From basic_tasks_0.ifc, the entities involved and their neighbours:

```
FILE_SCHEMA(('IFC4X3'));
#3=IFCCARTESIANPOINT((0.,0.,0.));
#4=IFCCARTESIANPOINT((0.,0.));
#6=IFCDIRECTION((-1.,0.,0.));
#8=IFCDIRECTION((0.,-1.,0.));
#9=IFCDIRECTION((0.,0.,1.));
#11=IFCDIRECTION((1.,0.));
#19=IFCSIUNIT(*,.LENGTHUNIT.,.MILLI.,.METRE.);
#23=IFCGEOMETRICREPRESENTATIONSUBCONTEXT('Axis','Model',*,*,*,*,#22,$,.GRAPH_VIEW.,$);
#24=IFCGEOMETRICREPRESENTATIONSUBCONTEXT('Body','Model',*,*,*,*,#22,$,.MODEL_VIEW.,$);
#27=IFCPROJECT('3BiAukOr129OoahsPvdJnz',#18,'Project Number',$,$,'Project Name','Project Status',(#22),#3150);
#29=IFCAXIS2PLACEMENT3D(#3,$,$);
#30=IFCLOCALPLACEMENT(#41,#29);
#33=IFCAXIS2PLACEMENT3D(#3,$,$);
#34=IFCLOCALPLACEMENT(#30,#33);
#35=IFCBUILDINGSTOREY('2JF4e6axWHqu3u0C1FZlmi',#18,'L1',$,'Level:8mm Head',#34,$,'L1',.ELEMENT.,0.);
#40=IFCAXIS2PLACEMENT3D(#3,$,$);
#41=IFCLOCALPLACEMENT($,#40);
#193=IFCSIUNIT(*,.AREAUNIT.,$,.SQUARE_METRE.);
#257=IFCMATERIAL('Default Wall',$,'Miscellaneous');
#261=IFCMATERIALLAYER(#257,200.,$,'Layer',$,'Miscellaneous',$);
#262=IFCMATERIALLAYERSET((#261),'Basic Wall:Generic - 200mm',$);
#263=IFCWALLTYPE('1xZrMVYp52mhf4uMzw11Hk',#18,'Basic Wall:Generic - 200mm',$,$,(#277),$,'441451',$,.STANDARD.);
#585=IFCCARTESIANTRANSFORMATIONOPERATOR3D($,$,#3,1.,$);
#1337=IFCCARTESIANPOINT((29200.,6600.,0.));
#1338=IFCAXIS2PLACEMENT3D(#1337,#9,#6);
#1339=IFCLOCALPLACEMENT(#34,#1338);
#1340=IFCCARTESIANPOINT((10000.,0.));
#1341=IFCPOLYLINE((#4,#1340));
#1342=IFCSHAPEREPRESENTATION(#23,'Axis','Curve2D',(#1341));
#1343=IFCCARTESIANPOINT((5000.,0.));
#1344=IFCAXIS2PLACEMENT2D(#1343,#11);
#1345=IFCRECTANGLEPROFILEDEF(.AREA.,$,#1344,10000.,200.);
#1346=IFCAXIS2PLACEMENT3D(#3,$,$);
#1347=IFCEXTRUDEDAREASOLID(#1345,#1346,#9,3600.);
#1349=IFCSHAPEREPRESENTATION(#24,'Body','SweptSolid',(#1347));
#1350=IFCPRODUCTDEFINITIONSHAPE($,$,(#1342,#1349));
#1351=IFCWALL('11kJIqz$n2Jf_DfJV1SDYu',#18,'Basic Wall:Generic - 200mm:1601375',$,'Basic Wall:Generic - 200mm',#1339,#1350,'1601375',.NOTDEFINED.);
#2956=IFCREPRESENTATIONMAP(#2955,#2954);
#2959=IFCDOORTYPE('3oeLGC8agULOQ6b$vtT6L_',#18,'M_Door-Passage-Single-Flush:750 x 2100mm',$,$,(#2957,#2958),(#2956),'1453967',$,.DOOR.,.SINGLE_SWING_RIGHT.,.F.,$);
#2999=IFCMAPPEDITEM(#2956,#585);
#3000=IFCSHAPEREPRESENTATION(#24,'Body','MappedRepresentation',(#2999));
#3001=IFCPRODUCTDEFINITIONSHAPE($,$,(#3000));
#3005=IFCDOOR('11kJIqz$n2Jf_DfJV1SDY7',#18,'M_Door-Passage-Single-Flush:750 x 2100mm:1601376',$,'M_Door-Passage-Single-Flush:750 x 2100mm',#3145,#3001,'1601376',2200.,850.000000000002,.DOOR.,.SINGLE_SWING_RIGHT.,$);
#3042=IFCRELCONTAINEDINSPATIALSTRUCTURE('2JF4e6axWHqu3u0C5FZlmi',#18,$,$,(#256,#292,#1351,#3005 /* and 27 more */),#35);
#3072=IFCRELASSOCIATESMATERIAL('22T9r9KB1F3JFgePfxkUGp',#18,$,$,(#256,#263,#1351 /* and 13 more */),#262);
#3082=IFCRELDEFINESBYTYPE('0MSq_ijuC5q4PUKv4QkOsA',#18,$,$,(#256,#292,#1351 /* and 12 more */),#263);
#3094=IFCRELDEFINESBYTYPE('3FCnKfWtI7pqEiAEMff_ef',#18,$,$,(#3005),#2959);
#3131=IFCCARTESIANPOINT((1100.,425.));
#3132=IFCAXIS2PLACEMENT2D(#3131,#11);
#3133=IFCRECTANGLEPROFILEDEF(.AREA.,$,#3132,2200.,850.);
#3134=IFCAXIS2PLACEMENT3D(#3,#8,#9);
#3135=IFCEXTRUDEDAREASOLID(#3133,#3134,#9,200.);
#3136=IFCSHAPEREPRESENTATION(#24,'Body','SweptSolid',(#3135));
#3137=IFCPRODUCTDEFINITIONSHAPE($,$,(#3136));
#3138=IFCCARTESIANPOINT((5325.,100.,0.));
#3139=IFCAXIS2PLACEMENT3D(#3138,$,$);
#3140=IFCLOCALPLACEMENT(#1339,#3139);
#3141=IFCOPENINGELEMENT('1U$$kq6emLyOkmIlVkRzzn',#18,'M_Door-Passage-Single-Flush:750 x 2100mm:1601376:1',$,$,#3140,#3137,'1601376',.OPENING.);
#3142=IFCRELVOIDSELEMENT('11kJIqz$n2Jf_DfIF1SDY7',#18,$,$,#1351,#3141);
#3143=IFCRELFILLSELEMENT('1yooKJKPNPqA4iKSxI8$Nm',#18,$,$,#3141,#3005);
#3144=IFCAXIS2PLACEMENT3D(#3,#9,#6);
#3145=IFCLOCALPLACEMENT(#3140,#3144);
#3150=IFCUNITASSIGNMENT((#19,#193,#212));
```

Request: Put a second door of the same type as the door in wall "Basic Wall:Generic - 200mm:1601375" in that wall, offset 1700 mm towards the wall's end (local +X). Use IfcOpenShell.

```python
import ifcopenshell
import ifcopenshell.api.feature
import ifcopenshell.api.geometry
import ifcopenshell.api.root
import ifcopenshell.geom
import ifcopenshell.util.element
import ifcopenshell.util.placement
import ifcopenshell.util.shape
import ifcopenshell.util.unit

model = ifcopenshell.open("basic_tasks_0.ifc")
unit_scale = ifcopenshell.util.unit.calculate_unit_scale(model)
settings = ifcopenshell.geom.settings()


def volume(element):
    """Net volume in cubic metres, openings subtracted."""
    shape = ifcopenshell.geom.create_shape(settings, element)
    return ifcopenshell.util.shape.get_volume(shape.geometry)


def reuse_history(source, copy):
    """copy_class also copies each property set's owner history, people and application; keep the originals."""
    for rel in copy.IsDefinedBy:
        if rel.is_a("IfcRelDefinesByProperties") and (history := rel.RelatingPropertyDefinition.OwnerHistory):
            rel.RelatingPropertyDefinition.OwnerHistory = source.OwnerHistory
            ifcopenshell.util.element.remove_deep2(model, history)


door = model.by_guid("11kJIqz$n2Jf_DfJV1SDY7")
opening = door.FillsVoids[0].RelatingOpeningElement
wall = opening.VoidsElements[0].RelatingBuildingElement
before = volume(wall)
shift = ifcopenshell.util.placement.get_local_placement(wall.ObjectPlacement)[:3, 0] * 1.7 / unit_scale

# copy_class copies the void relationship, type, container and properties, but no geometry.
new_opening = ifcopenshell.api.root.copy_class(model, product=opening)
new_opening.Representation = ifcopenshell.util.element.copy_deep(
    model, opening.Representation, exclude=["IfcGeometricRepresentationContext", "IfcRepresentationMap"]
)
new_opening.Name = "M_Door-Passage-Single-Flush:750 x 2100mm"
new_opening.Tag = None
new_door = ifcopenshell.api.root.copy_class(model, product=door)
new_door.Representation = ifcopenshell.util.element.copy_deep(
    model, door.Representation, exclude=["IfcGeometricRepresentationContext", "IfcRepresentationMap"]
)
new_door.Name = "M_Door-Passage-Single-Flush:750 x 2100mm"
new_door.Tag = None
reuse_history(door, new_door)
ifcopenshell.api.feature.add_filling(model, opening=new_opening, element=new_door)

for old, new in ((opening, new_opening), (door, new_door)):
    matrix = ifcopenshell.util.placement.get_local_placement(old.ObjectPlacement)
    matrix[:3, 3] += shift
    ifcopenshell.api.geometry.edit_object_placement(model, product=new, matrix=matrix, is_si=False)

after = volume(wall)

print(f"wall volume {before:.3f} -> {after:.3f} m3")

model.write("basic_tasks_0_v2.ifc")
```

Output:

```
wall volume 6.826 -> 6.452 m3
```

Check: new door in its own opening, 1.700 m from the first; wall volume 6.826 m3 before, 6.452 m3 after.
